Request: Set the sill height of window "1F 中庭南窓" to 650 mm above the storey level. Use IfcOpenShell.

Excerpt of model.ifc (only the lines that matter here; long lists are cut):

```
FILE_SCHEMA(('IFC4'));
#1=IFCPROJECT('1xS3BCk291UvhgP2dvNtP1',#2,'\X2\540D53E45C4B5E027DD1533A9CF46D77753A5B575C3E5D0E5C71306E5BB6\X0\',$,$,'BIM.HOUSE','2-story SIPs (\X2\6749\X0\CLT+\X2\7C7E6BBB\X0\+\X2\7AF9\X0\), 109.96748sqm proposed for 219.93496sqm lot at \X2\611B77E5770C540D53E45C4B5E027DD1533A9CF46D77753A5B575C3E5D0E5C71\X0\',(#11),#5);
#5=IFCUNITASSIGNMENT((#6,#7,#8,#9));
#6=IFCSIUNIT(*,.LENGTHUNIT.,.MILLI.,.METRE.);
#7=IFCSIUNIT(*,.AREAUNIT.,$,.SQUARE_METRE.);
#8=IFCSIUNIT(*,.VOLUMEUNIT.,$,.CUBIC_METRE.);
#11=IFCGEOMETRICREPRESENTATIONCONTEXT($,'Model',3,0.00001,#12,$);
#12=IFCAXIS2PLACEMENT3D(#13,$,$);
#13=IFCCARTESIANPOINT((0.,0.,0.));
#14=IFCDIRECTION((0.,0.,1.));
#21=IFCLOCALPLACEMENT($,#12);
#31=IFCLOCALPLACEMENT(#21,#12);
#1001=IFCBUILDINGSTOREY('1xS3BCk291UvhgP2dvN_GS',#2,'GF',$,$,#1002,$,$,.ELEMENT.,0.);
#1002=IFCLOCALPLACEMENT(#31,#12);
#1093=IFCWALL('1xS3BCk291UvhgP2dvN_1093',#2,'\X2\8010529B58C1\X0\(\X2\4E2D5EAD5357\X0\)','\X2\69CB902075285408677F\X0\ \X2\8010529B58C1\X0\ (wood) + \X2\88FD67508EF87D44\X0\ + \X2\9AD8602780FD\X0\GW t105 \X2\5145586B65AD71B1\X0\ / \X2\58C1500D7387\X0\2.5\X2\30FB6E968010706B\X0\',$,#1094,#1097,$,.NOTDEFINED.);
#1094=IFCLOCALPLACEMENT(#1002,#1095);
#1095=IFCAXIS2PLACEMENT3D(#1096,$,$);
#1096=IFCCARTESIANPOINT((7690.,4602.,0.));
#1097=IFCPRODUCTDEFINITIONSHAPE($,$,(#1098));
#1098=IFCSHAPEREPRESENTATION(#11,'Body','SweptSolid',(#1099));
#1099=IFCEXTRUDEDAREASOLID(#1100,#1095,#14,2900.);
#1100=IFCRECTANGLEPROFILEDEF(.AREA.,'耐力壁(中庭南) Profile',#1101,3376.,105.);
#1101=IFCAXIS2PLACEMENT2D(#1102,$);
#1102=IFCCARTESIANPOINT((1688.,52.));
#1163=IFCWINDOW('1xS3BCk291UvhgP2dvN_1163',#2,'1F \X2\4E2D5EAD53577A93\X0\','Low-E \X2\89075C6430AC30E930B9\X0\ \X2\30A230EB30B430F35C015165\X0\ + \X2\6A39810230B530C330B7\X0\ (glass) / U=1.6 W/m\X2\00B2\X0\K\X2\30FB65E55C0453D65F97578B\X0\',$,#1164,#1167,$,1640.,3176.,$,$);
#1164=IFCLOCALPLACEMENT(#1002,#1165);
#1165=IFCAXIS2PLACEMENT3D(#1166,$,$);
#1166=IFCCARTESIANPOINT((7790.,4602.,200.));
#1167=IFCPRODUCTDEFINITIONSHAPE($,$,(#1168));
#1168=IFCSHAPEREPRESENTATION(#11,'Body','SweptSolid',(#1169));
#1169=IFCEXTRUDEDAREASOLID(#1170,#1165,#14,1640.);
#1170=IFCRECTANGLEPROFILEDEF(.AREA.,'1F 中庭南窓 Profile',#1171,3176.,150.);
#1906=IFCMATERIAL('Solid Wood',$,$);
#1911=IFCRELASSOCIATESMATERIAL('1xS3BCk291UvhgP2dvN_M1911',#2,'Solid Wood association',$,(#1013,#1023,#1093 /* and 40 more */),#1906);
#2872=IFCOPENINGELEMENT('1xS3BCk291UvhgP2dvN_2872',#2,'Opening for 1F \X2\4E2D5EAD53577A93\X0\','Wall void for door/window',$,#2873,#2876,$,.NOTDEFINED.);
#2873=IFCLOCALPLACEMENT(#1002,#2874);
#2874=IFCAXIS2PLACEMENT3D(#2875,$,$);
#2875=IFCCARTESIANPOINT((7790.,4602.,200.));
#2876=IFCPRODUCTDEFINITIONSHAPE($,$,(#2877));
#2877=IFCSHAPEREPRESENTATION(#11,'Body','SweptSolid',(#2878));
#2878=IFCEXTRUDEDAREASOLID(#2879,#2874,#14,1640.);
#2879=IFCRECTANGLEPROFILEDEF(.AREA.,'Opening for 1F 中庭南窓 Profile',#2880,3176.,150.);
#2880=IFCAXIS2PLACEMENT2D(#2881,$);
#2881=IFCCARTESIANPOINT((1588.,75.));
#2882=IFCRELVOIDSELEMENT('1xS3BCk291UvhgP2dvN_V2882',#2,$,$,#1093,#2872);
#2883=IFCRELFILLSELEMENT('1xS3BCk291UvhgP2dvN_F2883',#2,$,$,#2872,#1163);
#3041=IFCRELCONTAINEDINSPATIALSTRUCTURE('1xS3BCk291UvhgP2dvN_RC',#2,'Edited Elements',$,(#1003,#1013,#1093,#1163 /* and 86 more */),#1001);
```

```python
import numpy as np
import ifcopenshell
import ifcopenshell.api.geometry
import ifcopenshell.geom
import ifcopenshell.util.element
import ifcopenshell.util.placement
import ifcopenshell.util.shape
import ifcopenshell.util.unit

model = ifcopenshell.open("model.ifc")
unit_scale = ifcopenshell.util.unit.calculate_unit_scale(model)

window = model.by_guid("1xS3BCk291UvhgP2dvN_1163")
opening = window.FillsVoids[0].RelatingOpeningElement
storey = ifcopenshell.util.element.get_container(window, ifc_class="IfcBuildingStorey")
level = ifcopenshell.util.placement.get_local_placement(storey.ObjectPlacement)[2, 3]

# The opening's origin need not be at the sill, so measure its lowest point.
shape = ifcopenshell.geom.create_shape(ifcopenshell.geom.settings(), opening)
bottom = ifcopenshell.util.shape.get_shape_bottom_elevation(shape, shape.geometry) / unit_scale
dz = level + 650.0 - bottom

shift = np.array([0.0, 0.0, dz])
# The window is not placed relative to its opening, so move both.
for product in (opening, window):
    matrix = ifcopenshell.util.placement.get_local_placement(product.ObjectPlacement)
    matrix[:3, 3] += shift
    ifcopenshell.api.geometry.edit_object_placement(model, product=product, matrix=matrix, is_si=False)

print(f"moved by {dz * unit_scale:+.3f} m")

model.write("model_updated.ifc")
```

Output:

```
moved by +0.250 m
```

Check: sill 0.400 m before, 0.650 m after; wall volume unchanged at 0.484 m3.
